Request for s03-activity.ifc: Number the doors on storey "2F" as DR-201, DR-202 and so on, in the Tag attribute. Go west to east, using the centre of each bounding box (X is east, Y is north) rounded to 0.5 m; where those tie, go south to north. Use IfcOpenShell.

First a look at what the model holds.

```python
import ifcopenshell
import ifcopenshell.util.element
import ifcopenshell.util.placement

model = ifcopenshell.open("s03-activity.ifc")
print(model.schema)
storey = next(s for s in model.by_type("IfcBuildingStorey") if s.Name == "2F")
doors = [e for e in ifcopenshell.util.element.get_decomposition(storey) if e.is_a("IfcDoor")]
for e in sorted(doors, key=lambda e: e.id()):
    origin = ifcopenshell.util.placement.get_local_placement(e.ObjectPlacement)[:3, 3]
    print(e.id(), e.Tag, e.Name, origin.round(2) + 0.0, sep=" | ")
```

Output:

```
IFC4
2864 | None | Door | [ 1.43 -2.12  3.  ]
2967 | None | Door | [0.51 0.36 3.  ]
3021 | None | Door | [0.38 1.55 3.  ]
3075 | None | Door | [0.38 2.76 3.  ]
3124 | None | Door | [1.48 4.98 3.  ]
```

```python
import ifcopenshell
import ifcopenshell.geom
import ifcopenshell.util.element
import ifcopenshell.util.shape

model = ifcopenshell.open("s03-activity.ifc")
settings = ifcopenshell.geom.settings()
settings.set("use-world-coords", True)


def centre(element):
    shape = ifcopenshell.geom.create_shape(settings, element)
    return ifcopenshell.util.shape.get_bbox_centroid(shape.geometry)


storey = next(s for s in model.by_type("IfcBuildingStorey") if s.Name == "2F")
doors = [e for e in ifcopenshell.util.element.get_decomposition(storey) if e.is_a("IfcDoor")]

# Insertion points can sit at a corner or the storey origin, so sort by the geometry (in metres).
centres = {e: centre(e) for e in doors}
doors.sort(key=lambda e: (round(centres[e][0] / 0.5), centres[e][1]))

for i, e in enumerate(doors, start=1):
    number = f"DR-2{i:02d}"
    e.Tag = number
    print(e.id(), number)

model.write("s03-activity_updated.ifc")
```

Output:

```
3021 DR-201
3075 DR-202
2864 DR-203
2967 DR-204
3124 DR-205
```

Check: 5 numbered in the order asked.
